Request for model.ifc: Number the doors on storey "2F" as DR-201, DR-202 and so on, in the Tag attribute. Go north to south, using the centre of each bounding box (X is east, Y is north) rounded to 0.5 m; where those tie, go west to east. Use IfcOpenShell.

First a look at what the model holds.

```python
import ifcopenshell
import ifcopenshell.util.element
import ifcopenshell.util.placement

model = ifcopenshell.open("model.ifc")
print(model.schema)
storey = next(s for s in model.by_type("IfcBuildingStorey") if s.Name == "2F")
doors = [e for e in ifcopenshell.util.element.get_decomposition(storey) if e.is_a("IfcDoor")]
for e in sorted(doors, key=lambda e: e.id()):
    origin = ifcopenshell.util.placement.get_local_placement(e.ObjectPlacement)[:3, 3]
    print(e.id(), e.Tag, e.Name, origin.round(2) + 0.0, sep=" | ")
```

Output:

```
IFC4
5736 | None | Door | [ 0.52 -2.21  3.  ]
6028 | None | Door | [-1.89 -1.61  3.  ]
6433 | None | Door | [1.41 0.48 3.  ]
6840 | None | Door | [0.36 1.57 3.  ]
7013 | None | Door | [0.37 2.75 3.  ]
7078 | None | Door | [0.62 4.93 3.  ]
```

```python
import ifcopenshell
import ifcopenshell.geom
import ifcopenshell.util.element
import ifcopenshell.util.shape

model = ifcopenshell.open("model.ifc")
settings = ifcopenshell.geom.settings()
settings.set("use-world-coords", True)


def centre(element):
    shape = ifcopenshell.geom.create_shape(settings, element)
    return ifcopenshell.util.shape.get_bbox_centroid(shape.geometry)


storey = next(s for s in model.by_type("IfcBuildingStorey") if s.Name == "2F")
doors = [e for e in ifcopenshell.util.element.get_decomposition(storey) if e.is_a("IfcDoor")]

# Insertion points can sit at a corner or the storey origin, so sort by the geometry (in metres).
centres = {e: centre(e) for e in doors}
doors.sort(key=lambda e: (-round(centres[e][1] / 0.5), centres[e][0]))

for i, e in enumerate(doors, start=1):
    number = f"DR-2{i:02d}"
    e.Tag = number
    print(e.id(), number)

model.write("model-out.ifc")
```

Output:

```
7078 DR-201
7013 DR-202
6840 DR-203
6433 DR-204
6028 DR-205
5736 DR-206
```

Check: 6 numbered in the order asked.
